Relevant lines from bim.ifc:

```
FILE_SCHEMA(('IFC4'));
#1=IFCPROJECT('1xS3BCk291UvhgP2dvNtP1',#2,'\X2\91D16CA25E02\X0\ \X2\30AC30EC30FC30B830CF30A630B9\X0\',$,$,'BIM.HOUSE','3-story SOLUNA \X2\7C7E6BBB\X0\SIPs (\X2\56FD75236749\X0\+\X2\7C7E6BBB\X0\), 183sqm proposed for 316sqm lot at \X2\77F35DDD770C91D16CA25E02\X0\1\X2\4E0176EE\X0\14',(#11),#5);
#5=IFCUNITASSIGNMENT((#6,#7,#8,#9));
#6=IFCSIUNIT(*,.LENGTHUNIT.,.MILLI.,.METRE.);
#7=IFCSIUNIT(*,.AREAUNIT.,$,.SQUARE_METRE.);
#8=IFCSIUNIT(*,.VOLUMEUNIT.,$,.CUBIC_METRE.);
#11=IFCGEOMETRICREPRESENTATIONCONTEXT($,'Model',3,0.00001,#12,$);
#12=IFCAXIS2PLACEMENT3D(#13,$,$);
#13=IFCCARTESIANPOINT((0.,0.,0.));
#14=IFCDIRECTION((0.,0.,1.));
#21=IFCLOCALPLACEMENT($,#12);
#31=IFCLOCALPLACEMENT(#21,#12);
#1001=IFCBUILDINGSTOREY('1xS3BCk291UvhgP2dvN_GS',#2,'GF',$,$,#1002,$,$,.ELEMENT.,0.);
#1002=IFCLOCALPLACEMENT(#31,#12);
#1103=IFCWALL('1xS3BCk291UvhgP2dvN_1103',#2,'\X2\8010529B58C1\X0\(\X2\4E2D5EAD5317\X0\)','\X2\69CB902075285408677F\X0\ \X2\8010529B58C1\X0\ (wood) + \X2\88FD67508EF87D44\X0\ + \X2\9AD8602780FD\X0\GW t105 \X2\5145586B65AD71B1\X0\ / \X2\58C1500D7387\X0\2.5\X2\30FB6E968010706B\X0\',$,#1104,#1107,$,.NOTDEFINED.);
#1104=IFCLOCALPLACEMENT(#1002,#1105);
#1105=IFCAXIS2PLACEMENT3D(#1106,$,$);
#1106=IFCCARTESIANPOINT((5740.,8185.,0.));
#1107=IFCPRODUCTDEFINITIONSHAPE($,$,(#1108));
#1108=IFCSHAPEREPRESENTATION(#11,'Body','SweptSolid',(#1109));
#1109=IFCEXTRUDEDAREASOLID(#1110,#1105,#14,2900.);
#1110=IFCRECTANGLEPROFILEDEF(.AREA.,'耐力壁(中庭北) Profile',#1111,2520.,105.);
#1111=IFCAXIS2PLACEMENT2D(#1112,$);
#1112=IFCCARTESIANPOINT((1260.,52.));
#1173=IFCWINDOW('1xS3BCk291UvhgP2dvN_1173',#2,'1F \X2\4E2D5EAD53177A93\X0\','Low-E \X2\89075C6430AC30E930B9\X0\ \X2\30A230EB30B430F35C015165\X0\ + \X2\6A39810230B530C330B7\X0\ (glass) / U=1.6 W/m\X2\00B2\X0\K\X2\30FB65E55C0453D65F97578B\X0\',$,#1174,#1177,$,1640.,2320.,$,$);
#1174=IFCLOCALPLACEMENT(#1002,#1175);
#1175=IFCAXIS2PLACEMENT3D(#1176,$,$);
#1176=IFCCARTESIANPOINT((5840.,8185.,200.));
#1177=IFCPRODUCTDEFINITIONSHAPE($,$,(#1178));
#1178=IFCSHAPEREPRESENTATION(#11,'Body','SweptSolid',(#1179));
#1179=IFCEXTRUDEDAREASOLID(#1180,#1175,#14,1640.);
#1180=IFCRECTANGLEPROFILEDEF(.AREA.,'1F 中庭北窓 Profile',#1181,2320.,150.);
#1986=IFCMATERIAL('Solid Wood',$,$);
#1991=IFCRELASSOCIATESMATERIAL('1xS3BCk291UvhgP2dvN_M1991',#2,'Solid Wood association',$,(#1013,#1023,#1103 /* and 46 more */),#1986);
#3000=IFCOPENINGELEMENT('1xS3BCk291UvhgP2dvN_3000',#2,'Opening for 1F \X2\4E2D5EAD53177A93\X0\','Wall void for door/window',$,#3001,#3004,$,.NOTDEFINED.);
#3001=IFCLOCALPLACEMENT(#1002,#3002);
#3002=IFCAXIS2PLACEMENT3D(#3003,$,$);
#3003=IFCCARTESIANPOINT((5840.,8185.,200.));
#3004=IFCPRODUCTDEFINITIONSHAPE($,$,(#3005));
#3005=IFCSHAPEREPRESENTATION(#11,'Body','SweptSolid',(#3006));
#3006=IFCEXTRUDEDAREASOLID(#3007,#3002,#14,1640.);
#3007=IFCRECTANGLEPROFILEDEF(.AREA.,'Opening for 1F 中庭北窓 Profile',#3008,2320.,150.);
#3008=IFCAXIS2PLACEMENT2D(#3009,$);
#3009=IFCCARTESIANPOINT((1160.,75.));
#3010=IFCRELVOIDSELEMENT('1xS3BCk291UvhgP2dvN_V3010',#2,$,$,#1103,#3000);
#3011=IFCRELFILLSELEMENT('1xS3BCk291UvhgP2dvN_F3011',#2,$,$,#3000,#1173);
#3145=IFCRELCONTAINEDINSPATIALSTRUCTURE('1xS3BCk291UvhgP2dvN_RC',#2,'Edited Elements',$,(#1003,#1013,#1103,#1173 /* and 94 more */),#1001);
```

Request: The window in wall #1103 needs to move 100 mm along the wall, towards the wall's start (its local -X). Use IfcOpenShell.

```python
import ifcopenshell
import ifcopenshell.api.geometry
import ifcopenshell.util.placement

model = ifcopenshell.open("bim.ifc")

window = model.by_guid("1xS3BCk291UvhgP2dvN_1173")
opening = window.FillsVoids[0].RelatingOpeningElement
wall = opening.VoidsElements[0].RelatingBuildingElement

wall_matrix = ifcopenshell.util.placement.get_local_placement(wall.ObjectPlacement)
shift = wall_matrix[:3, 0] * -100.0
before = ifcopenshell.util.placement.get_local_placement(window.ObjectPlacement)[:3, 3].copy()

# The window is not placed relative to its opening, so move both.
for product in (opening, window):
    matrix = ifcopenshell.util.placement.get_local_placement(product.ObjectPlacement)
    matrix[:3, 3] += shift
    ifcopenshell.api.geometry.edit_object_placement(model, product=product, matrix=matrix, is_si=False)

after = ifcopenshell.util.placement.get_local_placement(window.ObjectPlacement)[:3, 3]
print("window moved by", (after - before).round(3) + 0.0)

model.write("bim_v2.ifc")
```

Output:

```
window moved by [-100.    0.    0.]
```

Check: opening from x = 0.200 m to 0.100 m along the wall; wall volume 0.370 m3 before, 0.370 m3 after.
